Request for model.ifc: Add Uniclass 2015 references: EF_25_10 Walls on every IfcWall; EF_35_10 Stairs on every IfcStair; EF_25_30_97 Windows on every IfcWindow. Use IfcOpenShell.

First a look at what the model holds.

```python
import ifcopenshell

model = ifcopenshell.open("model.ifc")
print(model.schema)
print("classifications:", [c.Name for c in model.by_type("IfcClassification")])
for ifc_class in ("IfcDoor", "IfcRoof", "IfcStair", "IfcWall", "IfcWindow"):
    print(ifc_class, len(model.by_type(ifc_class)))
```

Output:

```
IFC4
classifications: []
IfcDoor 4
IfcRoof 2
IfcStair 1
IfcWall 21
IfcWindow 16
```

```python
import ifcopenshell
import ifcopenshell.api.classification

model = ifcopenshell.open("model.ifc")

system = ifcopenshell.api.classification.add_classification(model, classification="Uniclass 2015")

codes = {
    "IfcWall": ("EF_25_10", "Walls"),
    "IfcStair": ("EF_35_10", "Stairs"),
    "IfcWindow": ("EF_25_30_97", "Windows"),
}
for ifc_class, (code, name) in codes.items():
    products = model.by_type(ifc_class)
    ifcopenshell.api.classification.add_reference(
        model, products=products, classification=system, identification=code, name=name
    )
    print(code, len(products))

model.write("model_edited.ifc")
```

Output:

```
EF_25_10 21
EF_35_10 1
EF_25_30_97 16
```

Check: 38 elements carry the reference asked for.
